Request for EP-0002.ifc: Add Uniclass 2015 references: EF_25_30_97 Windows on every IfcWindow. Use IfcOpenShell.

First a look at what the model holds.

```python
import ifcopenshell

model = ifcopenshell.open("EP-0002.ifc")
print(model.schema)
print("classifications:", [c.Name for c in model.by_type("IfcClassification")])
for ifc_class in ("IfcDoor", "IfcRoof", "IfcStair", "IfcWall", "IfcWindow"):
    print(ifc_class, len(model.by_type(ifc_class)))
```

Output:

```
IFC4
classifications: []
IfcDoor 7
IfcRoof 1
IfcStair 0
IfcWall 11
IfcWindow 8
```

```python
import ifcopenshell
import ifcopenshell.api.classification

model = ifcopenshell.open("EP-0002.ifc")

system = ifcopenshell.api.classification.add_classification(model, classification="Uniclass 2015")

codes = {
    "IfcWindow": ("EF_25_30_97", "Windows"),
}
for ifc_class, (code, name) in codes.items():
    products = model.by_type(ifc_class)
    ifcopenshell.api.classification.add_reference(
        model, products=products, classification=system, identification=code, name=name
    )
    print(code, len(products))

model.write("EP-0002_rev.ifc")
```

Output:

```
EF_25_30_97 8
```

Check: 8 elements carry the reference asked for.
